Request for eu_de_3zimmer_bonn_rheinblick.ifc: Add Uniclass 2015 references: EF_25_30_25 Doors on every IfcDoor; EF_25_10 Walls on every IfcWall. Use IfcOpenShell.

First a look at what the model holds.

```python
import ifcopenshell

model = ifcopenshell.open("eu_de_3zimmer_bonn_rheinblick.ifc")
print(model.schema)
print("classifications:", [c.Name for c in model.by_type("IfcClassification")])
for ifc_class in ("IfcDoor", "IfcRoof", "IfcStair", "IfcWall", "IfcWindow"):
    print(ifc_class, len(model.by_type(ifc_class)))
```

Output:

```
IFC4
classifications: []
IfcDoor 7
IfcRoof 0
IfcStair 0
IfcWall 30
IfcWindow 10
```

```python
import ifcopenshell
import ifcopenshell.api.classification

model = ifcopenshell.open("eu_de_3zimmer_bonn_rheinblick.ifc")

system = ifcopenshell.api.classification.add_classification(model, classification="Uniclass 2015")

codes = {
    "IfcDoor": ("EF_25_30_25", "Doors"),
    "IfcWall": ("EF_25_10", "Walls"),
}
for ifc_class, (code, name) in codes.items():
    products = model.by_type(ifc_class)
    ifcopenshell.api.classification.add_reference(
        model, products=products, classification=system, identification=code, name=name
    )
    print(code, len(products))

model.write("eu_de_3zimmer_bonn_rheinblick_edited.ifc")
```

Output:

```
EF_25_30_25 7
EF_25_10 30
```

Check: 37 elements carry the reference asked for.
